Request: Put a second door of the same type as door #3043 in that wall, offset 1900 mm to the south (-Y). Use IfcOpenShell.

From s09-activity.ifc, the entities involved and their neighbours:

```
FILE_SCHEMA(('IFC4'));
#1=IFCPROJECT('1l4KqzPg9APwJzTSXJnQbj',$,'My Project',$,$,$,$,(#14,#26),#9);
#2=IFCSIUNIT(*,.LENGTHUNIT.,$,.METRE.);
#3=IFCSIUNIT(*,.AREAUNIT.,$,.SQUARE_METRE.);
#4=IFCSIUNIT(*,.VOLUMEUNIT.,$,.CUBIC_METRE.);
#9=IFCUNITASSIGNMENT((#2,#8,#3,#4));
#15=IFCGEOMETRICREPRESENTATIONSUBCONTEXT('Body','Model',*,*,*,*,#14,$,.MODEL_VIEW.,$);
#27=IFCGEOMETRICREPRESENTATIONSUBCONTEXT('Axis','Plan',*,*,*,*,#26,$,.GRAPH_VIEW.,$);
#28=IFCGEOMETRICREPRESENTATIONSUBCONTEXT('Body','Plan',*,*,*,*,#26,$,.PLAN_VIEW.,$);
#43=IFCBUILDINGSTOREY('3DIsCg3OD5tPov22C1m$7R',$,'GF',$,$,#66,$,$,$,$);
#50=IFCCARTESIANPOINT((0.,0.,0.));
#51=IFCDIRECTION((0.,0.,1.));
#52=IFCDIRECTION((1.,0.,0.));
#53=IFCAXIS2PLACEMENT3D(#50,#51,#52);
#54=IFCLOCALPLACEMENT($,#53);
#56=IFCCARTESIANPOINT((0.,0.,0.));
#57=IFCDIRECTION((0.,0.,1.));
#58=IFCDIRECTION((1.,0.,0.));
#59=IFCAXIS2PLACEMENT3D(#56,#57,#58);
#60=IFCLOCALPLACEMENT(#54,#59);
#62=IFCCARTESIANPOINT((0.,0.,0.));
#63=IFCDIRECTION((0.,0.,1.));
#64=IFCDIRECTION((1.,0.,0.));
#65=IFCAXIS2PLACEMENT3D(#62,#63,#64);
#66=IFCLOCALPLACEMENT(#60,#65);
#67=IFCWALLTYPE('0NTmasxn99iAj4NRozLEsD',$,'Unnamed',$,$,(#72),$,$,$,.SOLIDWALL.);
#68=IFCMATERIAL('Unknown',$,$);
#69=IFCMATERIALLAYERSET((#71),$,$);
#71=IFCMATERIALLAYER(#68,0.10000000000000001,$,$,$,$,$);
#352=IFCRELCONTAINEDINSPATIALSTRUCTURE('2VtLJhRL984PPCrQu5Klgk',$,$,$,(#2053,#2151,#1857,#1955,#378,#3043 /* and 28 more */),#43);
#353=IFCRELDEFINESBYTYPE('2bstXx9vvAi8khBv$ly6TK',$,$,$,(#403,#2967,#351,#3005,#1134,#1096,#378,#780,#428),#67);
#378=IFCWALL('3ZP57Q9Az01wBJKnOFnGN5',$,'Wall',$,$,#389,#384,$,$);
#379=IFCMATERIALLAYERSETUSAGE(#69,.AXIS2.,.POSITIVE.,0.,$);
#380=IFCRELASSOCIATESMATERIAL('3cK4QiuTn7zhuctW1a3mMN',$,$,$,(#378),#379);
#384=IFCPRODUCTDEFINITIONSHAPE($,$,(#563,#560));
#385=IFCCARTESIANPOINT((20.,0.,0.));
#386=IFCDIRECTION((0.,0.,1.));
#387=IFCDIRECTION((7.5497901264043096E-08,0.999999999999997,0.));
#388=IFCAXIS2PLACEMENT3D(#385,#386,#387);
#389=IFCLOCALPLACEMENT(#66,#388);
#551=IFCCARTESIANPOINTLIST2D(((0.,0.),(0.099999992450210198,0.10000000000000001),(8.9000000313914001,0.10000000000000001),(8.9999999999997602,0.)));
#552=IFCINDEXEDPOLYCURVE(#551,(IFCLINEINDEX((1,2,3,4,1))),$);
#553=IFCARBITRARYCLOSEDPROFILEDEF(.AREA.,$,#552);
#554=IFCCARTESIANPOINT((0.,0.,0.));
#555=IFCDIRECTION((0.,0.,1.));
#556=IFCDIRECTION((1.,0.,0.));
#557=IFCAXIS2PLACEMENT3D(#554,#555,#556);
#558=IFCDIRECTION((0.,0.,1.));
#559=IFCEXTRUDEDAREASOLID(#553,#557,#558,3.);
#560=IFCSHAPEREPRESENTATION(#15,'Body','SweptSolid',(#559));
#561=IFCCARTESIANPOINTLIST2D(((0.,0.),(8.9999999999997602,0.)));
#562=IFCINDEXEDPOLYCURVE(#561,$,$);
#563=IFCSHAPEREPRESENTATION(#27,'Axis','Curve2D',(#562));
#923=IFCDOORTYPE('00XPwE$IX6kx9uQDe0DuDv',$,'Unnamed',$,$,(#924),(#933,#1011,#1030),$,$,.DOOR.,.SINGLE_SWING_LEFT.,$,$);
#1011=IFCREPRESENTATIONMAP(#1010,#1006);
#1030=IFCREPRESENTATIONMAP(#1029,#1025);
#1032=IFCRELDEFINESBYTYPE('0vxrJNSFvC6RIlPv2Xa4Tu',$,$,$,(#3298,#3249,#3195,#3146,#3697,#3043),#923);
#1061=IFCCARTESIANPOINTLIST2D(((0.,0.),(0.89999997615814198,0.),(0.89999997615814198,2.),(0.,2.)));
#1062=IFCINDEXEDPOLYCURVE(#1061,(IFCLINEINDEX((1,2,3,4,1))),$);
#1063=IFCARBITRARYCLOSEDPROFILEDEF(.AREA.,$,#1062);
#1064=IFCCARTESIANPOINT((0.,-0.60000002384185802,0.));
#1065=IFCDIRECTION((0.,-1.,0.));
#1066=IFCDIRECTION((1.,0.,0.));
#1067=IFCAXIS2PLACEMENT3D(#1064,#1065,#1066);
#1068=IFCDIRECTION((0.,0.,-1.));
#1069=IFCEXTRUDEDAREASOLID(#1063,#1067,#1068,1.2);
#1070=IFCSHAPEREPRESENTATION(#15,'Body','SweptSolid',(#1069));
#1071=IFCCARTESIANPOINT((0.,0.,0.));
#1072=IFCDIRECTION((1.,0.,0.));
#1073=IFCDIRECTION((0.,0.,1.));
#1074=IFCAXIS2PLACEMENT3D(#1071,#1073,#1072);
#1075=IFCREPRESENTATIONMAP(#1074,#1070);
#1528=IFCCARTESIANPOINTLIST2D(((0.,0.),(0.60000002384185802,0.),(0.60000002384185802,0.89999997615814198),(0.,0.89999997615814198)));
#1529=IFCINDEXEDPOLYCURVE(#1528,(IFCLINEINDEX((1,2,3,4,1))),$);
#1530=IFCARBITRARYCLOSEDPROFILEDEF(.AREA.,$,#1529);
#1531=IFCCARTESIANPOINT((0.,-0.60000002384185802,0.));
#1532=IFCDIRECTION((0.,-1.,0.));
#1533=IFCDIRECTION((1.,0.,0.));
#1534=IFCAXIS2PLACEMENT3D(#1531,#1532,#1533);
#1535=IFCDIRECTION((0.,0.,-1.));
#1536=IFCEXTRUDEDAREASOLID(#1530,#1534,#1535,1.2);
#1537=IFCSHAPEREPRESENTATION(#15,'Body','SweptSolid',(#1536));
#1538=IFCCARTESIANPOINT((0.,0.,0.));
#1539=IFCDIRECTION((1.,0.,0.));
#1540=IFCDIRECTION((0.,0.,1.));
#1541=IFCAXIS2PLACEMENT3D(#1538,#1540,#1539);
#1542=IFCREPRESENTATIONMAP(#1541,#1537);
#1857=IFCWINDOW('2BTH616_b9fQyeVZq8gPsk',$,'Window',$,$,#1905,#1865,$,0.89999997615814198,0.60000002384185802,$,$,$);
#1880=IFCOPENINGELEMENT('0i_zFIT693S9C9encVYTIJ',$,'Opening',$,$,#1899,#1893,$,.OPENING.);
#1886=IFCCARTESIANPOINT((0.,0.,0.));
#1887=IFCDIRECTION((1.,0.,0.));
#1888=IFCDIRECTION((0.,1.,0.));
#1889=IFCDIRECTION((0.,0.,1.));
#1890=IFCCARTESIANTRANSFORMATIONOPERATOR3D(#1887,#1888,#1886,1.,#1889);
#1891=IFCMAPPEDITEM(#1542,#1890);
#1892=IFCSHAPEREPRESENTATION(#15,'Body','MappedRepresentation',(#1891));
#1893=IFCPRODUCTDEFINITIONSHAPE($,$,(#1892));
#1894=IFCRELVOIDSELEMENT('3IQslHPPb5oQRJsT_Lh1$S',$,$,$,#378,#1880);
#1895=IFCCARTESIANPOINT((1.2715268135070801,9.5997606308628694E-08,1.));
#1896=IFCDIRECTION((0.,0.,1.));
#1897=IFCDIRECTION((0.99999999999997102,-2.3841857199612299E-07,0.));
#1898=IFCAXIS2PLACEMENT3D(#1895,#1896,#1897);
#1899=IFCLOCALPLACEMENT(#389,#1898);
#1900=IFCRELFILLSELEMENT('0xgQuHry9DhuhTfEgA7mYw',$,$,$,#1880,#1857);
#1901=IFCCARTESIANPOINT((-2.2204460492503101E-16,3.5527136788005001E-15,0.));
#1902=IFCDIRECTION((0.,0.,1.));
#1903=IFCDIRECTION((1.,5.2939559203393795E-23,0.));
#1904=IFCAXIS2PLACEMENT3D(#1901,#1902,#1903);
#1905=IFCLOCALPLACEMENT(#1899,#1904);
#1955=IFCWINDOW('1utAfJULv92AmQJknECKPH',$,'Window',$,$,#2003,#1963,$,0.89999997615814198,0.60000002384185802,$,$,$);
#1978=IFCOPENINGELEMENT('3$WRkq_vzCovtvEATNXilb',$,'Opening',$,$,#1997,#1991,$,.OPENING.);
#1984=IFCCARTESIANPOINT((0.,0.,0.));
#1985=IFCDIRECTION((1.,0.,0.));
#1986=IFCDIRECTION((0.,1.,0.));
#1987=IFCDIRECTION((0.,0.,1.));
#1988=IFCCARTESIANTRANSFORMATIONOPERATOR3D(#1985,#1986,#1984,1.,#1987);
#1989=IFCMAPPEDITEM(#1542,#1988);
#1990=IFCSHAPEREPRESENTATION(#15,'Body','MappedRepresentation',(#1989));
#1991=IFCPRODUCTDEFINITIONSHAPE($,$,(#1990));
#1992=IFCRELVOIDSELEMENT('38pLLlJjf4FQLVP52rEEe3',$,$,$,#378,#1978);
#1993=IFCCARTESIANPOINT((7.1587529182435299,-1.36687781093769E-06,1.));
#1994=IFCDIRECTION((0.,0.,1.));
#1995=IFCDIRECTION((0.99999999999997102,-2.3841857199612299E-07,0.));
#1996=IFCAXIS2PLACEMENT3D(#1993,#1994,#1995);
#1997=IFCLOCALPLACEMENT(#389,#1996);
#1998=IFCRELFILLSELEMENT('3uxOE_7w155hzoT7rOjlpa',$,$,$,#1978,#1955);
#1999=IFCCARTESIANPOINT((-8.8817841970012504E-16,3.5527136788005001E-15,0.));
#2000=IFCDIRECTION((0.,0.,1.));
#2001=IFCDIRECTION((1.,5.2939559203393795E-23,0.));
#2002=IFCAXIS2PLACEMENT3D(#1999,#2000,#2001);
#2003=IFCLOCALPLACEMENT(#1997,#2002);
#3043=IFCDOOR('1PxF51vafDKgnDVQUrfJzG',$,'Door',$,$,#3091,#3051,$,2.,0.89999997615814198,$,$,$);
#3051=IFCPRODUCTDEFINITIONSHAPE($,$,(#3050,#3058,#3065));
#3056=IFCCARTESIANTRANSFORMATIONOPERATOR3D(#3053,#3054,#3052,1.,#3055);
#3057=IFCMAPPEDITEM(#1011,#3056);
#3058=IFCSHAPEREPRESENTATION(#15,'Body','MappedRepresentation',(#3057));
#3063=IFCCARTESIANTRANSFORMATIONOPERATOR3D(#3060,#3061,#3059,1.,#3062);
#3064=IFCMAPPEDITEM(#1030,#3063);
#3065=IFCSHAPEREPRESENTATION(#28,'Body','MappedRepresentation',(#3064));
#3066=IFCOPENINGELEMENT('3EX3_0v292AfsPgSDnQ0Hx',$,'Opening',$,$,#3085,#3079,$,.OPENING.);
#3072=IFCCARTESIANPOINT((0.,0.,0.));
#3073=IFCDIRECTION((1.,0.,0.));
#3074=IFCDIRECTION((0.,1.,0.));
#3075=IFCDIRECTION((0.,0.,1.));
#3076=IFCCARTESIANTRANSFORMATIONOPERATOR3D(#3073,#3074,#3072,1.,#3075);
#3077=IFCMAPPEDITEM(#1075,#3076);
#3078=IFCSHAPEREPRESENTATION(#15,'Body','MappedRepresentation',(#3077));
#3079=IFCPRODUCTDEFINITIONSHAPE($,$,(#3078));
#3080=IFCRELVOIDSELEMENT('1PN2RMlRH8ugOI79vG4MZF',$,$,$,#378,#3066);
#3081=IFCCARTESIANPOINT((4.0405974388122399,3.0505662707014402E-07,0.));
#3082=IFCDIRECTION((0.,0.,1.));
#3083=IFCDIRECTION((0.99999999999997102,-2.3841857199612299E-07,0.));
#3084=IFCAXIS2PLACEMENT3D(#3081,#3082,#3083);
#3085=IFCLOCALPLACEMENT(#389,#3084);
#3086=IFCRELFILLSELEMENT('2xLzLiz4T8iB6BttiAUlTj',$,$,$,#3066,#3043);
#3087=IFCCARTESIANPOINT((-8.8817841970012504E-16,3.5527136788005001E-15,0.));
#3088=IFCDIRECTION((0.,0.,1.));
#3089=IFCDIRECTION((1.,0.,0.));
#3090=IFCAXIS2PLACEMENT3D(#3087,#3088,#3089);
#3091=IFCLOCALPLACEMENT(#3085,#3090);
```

```python
import ifcopenshell
import ifcopenshell.api.feature
import ifcopenshell.api.geometry
import ifcopenshell.api.root
import ifcopenshell.geom
import ifcopenshell.util.element
import ifcopenshell.util.placement
import ifcopenshell.util.shape
import ifcopenshell.util.unit

model = ifcopenshell.open("s09-activity.ifc")
unit_scale = ifcopenshell.util.unit.calculate_unit_scale(model)
settings = ifcopenshell.geom.settings()


def volume(element):
    """Net volume in cubic metres, openings subtracted."""
    shape = ifcopenshell.geom.create_shape(settings, element)
    return ifcopenshell.util.shape.get_volume(shape.geometry)


door = model.by_id(3043)
opening = door.FillsVoids[0].RelatingOpeningElement
wall = opening.VoidsElements[0].RelatingBuildingElement
before = volume(wall)
shift = ifcopenshell.util.placement.get_local_placement(wall.ObjectPlacement)[:3, 0] * -1.9 / unit_scale

# copy_class copies the void relationship, type, container and properties, but no geometry.
new_opening = ifcopenshell.api.root.copy_class(model, product=opening)
new_opening.Representation = ifcopenshell.util.element.copy_deep(
    model, opening.Representation, exclude=["IfcGeometricRepresentationContext", "IfcRepresentationMap"]
)
new_door = ifcopenshell.api.root.copy_class(model, product=door)
new_door.Representation = ifcopenshell.util.element.copy_deep(
    model, door.Representation, exclude=["IfcGeometricRepresentationContext", "IfcRepresentationMap"]
)
ifcopenshell.api.feature.add_filling(model, opening=new_opening, element=new_door)

for old, new in ((opening, new_opening), (door, new_door)):
    matrix = ifcopenshell.util.placement.get_local_placement(old.ObjectPlacement)
    matrix[:3, 3] += shift
    ifcopenshell.api.geometry.edit_object_placement(model, product=new, matrix=matrix, is_si=False)

after = volume(wall)

print(f"wall volume {before:.3f} -> {after:.3f} m3")

model.write("s09-activity_edited.ifc")
```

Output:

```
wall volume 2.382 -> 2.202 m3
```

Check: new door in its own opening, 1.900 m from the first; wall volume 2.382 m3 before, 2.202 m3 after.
